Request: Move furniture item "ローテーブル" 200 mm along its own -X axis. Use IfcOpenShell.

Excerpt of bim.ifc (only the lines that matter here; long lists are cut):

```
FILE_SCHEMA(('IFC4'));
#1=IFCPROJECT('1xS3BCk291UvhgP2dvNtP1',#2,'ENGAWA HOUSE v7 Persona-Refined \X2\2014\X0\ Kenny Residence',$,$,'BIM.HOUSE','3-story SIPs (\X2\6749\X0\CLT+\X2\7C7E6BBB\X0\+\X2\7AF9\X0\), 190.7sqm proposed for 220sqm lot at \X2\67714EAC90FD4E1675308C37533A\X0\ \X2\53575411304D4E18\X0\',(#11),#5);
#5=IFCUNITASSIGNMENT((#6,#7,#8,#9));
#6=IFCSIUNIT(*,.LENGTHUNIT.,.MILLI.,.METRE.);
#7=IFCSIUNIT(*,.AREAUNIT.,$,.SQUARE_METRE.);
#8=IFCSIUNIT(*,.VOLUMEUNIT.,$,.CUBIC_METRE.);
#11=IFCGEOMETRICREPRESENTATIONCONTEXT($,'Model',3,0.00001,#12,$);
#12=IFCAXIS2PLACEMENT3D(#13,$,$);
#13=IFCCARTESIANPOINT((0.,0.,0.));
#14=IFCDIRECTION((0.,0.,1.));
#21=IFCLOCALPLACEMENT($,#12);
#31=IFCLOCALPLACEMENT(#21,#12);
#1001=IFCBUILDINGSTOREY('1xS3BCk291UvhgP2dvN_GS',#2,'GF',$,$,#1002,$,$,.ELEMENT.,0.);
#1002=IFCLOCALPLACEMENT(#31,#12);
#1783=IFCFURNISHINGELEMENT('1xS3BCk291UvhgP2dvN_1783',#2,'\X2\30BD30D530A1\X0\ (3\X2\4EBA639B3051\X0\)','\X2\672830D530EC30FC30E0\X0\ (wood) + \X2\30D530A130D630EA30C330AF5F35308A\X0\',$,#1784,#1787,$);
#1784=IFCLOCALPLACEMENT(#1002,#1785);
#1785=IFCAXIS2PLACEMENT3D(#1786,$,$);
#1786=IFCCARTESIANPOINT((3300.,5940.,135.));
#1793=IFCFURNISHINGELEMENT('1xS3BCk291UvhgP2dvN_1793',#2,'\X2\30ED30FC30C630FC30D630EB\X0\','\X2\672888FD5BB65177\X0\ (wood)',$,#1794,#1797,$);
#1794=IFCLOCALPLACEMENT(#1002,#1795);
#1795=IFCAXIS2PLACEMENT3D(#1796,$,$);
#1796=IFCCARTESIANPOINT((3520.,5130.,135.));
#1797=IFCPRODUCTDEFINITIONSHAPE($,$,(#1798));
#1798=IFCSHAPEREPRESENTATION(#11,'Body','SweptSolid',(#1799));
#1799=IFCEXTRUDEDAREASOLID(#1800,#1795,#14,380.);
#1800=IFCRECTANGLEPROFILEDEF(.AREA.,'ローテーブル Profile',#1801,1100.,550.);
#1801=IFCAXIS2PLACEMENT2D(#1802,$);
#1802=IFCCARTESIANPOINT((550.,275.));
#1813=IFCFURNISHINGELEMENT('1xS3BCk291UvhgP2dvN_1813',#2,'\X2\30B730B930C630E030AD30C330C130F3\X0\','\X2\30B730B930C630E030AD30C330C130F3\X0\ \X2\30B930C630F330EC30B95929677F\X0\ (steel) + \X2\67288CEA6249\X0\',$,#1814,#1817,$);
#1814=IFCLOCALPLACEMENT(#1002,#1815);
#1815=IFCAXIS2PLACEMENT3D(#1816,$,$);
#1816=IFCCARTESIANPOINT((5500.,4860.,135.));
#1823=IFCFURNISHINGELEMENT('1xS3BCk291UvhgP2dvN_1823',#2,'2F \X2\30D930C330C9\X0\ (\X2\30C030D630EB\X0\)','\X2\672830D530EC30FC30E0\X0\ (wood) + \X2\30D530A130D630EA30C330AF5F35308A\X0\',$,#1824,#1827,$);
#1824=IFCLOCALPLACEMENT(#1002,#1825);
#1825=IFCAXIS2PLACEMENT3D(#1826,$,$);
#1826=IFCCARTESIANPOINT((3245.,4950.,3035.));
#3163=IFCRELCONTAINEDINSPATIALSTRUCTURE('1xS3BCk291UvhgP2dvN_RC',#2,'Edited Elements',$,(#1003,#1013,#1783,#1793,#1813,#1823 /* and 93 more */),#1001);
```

```python
import ifcopenshell
import ifcopenshell.api.geometry
import ifcopenshell.util.placement
import ifcopenshell.util.unit

model = ifcopenshell.open("bim.ifc")
unit_scale = ifcopenshell.util.unit.calculate_unit_scale(model)

item = model.by_guid("1xS3BCk291UvhgP2dvN_1793")
matrix = ifcopenshell.util.placement.get_local_placement(item.ObjectPlacement)
matrix[:3, 3] -= matrix[:3, 0] * 0.2 / unit_scale
ifcopenshell.api.geometry.edit_object_placement(model, product=item, matrix=matrix, is_si=False)

print(ifcopenshell.util.placement.get_local_placement(item.ObjectPlacement).round(3) + 0.0)

model.write("bim_edited.ifc")
```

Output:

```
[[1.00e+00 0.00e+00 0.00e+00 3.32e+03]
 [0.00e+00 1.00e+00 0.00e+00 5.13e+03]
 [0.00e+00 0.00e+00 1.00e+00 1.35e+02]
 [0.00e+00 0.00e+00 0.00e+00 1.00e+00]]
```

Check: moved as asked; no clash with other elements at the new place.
